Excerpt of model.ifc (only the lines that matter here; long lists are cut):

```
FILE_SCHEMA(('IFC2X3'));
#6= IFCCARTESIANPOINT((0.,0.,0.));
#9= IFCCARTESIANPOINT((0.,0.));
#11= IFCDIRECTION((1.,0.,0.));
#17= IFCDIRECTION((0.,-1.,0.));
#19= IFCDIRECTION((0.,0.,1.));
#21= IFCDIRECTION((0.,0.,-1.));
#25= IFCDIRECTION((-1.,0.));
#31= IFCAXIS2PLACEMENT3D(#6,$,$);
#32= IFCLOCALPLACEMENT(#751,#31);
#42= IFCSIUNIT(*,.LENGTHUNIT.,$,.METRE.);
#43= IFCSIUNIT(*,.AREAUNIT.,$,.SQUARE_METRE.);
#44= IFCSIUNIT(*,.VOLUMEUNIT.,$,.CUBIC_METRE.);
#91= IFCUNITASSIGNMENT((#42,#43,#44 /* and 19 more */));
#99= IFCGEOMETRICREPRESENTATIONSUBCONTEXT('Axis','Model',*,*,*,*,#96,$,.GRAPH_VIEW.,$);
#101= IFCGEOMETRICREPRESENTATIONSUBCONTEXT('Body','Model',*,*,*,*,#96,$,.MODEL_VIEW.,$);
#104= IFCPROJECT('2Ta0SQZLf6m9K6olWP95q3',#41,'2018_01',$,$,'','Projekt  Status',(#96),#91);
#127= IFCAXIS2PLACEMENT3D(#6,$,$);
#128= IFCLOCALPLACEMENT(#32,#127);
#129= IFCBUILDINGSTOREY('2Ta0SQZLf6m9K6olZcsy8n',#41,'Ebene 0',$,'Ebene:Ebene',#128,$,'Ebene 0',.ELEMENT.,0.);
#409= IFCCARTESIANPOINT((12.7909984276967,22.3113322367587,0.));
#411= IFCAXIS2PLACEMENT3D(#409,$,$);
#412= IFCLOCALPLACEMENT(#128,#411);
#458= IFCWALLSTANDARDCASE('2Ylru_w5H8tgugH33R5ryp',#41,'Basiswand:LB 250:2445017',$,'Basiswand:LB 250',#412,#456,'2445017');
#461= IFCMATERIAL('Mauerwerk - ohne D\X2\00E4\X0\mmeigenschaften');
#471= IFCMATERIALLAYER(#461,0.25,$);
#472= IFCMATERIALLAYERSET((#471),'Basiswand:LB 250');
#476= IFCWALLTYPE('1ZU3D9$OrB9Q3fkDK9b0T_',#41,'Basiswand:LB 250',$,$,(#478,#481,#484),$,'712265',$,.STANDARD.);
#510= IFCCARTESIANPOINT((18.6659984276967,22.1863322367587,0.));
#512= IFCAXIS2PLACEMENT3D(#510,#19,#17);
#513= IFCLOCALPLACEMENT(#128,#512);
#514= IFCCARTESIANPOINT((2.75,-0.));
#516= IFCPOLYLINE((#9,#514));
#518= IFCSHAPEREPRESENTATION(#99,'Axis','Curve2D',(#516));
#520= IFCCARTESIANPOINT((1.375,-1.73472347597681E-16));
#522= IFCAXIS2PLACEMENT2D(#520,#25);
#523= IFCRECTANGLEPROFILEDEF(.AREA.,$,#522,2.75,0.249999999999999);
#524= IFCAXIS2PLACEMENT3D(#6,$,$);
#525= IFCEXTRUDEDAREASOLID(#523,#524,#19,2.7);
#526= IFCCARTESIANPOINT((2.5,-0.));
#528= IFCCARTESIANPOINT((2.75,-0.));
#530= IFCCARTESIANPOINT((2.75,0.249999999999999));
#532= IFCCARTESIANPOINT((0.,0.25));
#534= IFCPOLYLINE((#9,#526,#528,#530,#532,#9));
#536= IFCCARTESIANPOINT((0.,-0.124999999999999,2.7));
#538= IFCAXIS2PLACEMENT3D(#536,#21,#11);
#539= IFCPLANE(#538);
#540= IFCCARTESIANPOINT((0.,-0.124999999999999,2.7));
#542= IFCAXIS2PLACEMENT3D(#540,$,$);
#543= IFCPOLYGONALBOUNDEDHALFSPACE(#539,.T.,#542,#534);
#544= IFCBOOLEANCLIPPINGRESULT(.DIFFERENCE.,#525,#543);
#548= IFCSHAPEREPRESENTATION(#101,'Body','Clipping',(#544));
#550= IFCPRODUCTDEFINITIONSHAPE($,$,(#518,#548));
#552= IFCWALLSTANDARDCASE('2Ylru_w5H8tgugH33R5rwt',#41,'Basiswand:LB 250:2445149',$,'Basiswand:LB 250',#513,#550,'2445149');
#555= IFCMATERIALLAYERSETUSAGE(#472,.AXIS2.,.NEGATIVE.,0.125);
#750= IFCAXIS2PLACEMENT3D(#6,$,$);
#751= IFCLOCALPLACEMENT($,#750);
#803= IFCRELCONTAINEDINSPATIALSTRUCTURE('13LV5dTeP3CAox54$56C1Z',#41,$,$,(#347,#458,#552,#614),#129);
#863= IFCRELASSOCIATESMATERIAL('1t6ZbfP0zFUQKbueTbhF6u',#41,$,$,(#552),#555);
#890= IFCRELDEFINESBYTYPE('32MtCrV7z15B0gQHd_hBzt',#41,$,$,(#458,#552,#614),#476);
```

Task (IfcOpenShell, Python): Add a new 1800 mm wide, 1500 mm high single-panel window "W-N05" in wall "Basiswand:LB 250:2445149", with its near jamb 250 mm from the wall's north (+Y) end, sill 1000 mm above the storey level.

```python
import numpy as np
import ifcopenshell
import ifcopenshell.api.feature
import ifcopenshell.api.geometry
import ifcopenshell.api.root
import ifcopenshell.api.spatial
import ifcopenshell.api.type
import ifcopenshell.geom
import ifcopenshell.util.element
import ifcopenshell.util.placement
import ifcopenshell.util.representation
import ifcopenshell.util.shape
import ifcopenshell.util.unit

model = ifcopenshell.open("model.ifc")
unit_scale = ifcopenshell.util.unit.calculate_unit_scale(model)
settings = ifcopenshell.geom.settings()


def volume(element):
    """Net volume in cubic metres, openings subtracted."""
    shape = ifcopenshell.geom.create_shape(settings, element)
    return ifcopenshell.util.shape.get_volume(shape.geometry)


wall = model.by_guid("2Ylru_w5H8tgugH33R5rwt")
storey = ifcopenshell.util.element.get_container(wall, ifc_class="IfcBuildingStorey")
context = ifcopenshell.util.representation.get_context(model, "Model", "Body", "MODEL_VIEW")
before = volume(wall)

width, height, from_end, sill = 1.8, 1.5, 0.25, 1  # metres

# The wall runs along its own X axis, and the end named is its -X end.
wall_shape = ifcopenshell.geom.create_shape(settings, wall)
x, y, z = ifcopenshell.util.shape.get_vertices(wall_shape.geometry).T
start = x.min() + from_end
face, thickness = float(y.min()), float(y.max() - y.min())
wall_matrix = ifcopenshell.util.placement.get_local_placement(wall.ObjectPlacement)
level = ifcopenshell.util.placement.get_local_placement(storey.ObjectPlacement)[2, 3]


def in_wall(x, y):
    """Placement at x, y metres in the wall's axes, at sill height."""
    matrix = wall_matrix.copy()
    matrix[:, 3] = wall_matrix @ np.array([x / unit_scale, y / unit_scale, 0.0, 1.0])
    matrix[2, 3] = level + sill / unit_scale
    return matrix


# Opening: a box that overshoots both wall faces by 50 mm.
opening = ifcopenshell.api.root.create_entity(model, ifc_class="IfcOpeningElement")
box = ifcopenshell.api.geometry.add_wall_representation(
    model, context=context, length=width, height=height, thickness=thickness + 0.1
)
ifcopenshell.api.geometry.assign_representation(model, product=opening, representation=box)
ifcopenshell.api.geometry.edit_object_placement(model, product=opening, matrix=in_wall(start, face - 0.05), is_si=False)
ifcopenshell.api.feature.add_feature(model, feature=opening, element=wall)

window = ifcopenshell.api.root.create_entity(model, ifc_class="IfcWindow", name="W-N05")
window.OverallWidth, window.OverallHeight = width / unit_scale, height / unit_scale
body = ifcopenshell.api.geometry.add_window_representation(
    model,
    context=context,
    overall_width=window.OverallWidth,
    overall_height=window.OverallHeight,
    partition_type="SINGLE_PANEL",
)
ifcopenshell.api.geometry.assign_representation(model, product=window, representation=body)
ifcopenshell.api.spatial.assign_container(model, products=[window], relating_structure=storey)
fills = ifcopenshell.api.feature.add_filling(model, opening=opening, element=window)
fills.OwnerHistory = window.OwnerHistory  # required in IFC2X3

# IFC2X3 keeps the operation on the window style.
style = ifcopenshell.api.root.create_entity(model, ifc_class="IfcWindowStyle", name="W-N05")
style.OperationType, style.ConstructionType = "SINGLE_PANEL", "NOTDEFINED"
style.ParameterTakesPrecedence = style.Sizeable = False
ifcopenshell.api.type.assign_type(model, related_objects=[window], relating_type=style)

# Centre the window in the wall's thickness.
ifcopenshell.api.geometry.edit_object_placement(model, product=window, matrix=in_wall(start, face), is_si=False)
window_shape = ifcopenshell.geom.create_shape(settings, window)
depth = ifcopenshell.util.shape.get_vertices(window_shape.geometry)[:, 1]
offset = face + thickness / 2 - (depth.min() + depth.max()) / 2
ifcopenshell.api.geometry.edit_object_placement(model, product=window, matrix=in_wall(start, offset), is_si=False)

after = volume(wall)

print(f"wall volume {before:.3f} -> {after:.3f} m3")

model.write("model_edited.ifc")
```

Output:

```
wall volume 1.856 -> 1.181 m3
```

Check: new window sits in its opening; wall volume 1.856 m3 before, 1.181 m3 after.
